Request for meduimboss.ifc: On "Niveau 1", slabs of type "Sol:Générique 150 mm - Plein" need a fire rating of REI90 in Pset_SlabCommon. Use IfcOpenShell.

First a look at what the model holds.

```python
import ifcopenshell
import ifcopenshell.util.element

model = ifcopenshell.open("meduimboss.ifc")
print(model.schema)
storey = next(s for s in model.by_type("IfcBuildingStorey") if s.Name == "Niveau 1")
slabs = [e for e in ifcopenshell.util.element.get_decomposition(storey) if e.is_a("IfcSlab")]
seen = {}
for e in slabs:
    element_type = ifcopenshell.util.element.get_type(e)
    key = (element_type.Name if element_type != e and element_type else None, ifcopenshell.util.element.get_pset(e, "Pset_SlabCommon", "FireRating"))
    seen[key] = seen.get(key, 0) + 1
for (name, value), count in sorted(seen.items(), key=str):
    print(count, "x", name, "|", value)
```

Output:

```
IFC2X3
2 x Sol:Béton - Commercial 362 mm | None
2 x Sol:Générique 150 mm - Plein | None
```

```python
import ifcopenshell
import ifcopenshell.api.pset
import ifcopenshell.util.element

model = ifcopenshell.open("meduimboss.ifc")

storey = next(s for s in model.by_type("IfcBuildingStorey") if s.Name == "Niveau 1")
slabs = [e for e in ifcopenshell.util.element.get_decomposition(storey) if e.is_a("IfcSlab")]

count = 0
for e in slabs:
    element_type = ifcopenshell.util.element.get_type(e)
    if element_type in (None, e) or element_type.Name != "Sol:Générique 150 mm - Plein":
        continue
    # add_pset returns the element's existing set when there is one.
    pset = ifcopenshell.api.pset.add_pset(model, product=e, name="Pset_SlabCommon")
    ifcopenshell.api.pset.edit_pset(model, pset=pset, properties={"FireRating": "REI90"})
    count += 1

print(count, "slabs updated")

model.write("meduimboss_updated.ifc")
```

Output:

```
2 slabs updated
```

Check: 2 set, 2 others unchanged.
